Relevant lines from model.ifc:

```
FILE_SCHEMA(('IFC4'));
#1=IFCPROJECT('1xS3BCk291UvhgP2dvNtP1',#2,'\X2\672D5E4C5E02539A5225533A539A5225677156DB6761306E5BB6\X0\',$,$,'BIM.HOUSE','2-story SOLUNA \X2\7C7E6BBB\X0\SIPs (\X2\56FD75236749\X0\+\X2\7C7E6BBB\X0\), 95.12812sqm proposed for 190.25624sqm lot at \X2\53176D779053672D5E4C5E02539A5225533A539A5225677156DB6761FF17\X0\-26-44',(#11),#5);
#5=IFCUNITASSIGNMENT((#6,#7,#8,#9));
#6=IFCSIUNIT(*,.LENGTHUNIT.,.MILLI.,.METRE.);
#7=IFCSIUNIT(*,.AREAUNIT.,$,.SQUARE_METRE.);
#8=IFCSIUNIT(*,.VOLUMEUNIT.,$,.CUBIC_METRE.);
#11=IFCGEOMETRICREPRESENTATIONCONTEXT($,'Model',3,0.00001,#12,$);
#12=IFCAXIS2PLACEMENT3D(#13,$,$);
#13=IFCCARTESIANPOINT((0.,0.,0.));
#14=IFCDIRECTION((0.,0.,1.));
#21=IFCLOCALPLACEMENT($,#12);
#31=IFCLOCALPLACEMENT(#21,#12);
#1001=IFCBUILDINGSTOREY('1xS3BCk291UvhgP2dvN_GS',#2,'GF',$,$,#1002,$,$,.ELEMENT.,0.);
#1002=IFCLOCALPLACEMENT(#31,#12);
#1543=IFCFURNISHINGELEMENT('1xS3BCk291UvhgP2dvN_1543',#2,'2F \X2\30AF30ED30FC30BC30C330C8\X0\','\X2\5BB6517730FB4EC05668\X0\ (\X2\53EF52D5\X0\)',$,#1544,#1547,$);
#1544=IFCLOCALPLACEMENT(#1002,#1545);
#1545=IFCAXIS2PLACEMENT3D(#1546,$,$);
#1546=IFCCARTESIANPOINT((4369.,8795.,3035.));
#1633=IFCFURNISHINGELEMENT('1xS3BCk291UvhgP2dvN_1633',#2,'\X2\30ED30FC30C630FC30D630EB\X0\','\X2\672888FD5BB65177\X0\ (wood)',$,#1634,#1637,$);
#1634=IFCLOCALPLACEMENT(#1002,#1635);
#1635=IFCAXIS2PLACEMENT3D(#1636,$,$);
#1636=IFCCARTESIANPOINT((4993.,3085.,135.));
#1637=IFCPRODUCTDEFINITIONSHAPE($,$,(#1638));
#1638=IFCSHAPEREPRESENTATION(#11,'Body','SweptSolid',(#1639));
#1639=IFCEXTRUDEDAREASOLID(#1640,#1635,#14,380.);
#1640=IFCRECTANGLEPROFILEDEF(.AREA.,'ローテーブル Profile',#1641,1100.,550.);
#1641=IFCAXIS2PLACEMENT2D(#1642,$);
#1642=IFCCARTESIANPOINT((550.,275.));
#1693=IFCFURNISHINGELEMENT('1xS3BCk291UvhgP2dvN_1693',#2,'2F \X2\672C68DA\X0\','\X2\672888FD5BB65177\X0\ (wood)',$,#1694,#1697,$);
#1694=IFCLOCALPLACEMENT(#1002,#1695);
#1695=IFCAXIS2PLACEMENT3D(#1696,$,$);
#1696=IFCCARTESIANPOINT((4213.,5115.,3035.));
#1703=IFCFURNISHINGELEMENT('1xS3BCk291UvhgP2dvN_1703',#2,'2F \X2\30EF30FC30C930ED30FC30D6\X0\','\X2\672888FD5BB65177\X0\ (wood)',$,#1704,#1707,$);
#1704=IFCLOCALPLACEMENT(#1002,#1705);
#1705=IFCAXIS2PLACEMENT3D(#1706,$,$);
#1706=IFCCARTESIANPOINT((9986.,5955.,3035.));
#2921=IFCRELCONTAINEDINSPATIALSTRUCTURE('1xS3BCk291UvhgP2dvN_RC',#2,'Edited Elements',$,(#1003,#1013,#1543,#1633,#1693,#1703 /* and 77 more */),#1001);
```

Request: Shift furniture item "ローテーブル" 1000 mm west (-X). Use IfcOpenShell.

```python
import ifcopenshell
import ifcopenshell.api.geometry
import ifcopenshell.util.placement

model = ifcopenshell.open("model.ifc")

item = model.by_id(1633)
matrix = ifcopenshell.util.placement.get_local_placement(item.ObjectPlacement)
matrix[0, 3] -= 1000.0
ifcopenshell.api.geometry.edit_object_placement(model, product=item, matrix=matrix, is_si=False)

print(ifcopenshell.util.placement.get_local_placement(item.ObjectPlacement).round(3) + 0.0)

model.write("model-out.ifc")
```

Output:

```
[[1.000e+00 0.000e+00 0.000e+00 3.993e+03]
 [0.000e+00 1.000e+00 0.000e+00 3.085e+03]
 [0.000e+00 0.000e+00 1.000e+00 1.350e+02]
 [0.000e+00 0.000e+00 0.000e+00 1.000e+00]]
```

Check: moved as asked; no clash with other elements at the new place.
